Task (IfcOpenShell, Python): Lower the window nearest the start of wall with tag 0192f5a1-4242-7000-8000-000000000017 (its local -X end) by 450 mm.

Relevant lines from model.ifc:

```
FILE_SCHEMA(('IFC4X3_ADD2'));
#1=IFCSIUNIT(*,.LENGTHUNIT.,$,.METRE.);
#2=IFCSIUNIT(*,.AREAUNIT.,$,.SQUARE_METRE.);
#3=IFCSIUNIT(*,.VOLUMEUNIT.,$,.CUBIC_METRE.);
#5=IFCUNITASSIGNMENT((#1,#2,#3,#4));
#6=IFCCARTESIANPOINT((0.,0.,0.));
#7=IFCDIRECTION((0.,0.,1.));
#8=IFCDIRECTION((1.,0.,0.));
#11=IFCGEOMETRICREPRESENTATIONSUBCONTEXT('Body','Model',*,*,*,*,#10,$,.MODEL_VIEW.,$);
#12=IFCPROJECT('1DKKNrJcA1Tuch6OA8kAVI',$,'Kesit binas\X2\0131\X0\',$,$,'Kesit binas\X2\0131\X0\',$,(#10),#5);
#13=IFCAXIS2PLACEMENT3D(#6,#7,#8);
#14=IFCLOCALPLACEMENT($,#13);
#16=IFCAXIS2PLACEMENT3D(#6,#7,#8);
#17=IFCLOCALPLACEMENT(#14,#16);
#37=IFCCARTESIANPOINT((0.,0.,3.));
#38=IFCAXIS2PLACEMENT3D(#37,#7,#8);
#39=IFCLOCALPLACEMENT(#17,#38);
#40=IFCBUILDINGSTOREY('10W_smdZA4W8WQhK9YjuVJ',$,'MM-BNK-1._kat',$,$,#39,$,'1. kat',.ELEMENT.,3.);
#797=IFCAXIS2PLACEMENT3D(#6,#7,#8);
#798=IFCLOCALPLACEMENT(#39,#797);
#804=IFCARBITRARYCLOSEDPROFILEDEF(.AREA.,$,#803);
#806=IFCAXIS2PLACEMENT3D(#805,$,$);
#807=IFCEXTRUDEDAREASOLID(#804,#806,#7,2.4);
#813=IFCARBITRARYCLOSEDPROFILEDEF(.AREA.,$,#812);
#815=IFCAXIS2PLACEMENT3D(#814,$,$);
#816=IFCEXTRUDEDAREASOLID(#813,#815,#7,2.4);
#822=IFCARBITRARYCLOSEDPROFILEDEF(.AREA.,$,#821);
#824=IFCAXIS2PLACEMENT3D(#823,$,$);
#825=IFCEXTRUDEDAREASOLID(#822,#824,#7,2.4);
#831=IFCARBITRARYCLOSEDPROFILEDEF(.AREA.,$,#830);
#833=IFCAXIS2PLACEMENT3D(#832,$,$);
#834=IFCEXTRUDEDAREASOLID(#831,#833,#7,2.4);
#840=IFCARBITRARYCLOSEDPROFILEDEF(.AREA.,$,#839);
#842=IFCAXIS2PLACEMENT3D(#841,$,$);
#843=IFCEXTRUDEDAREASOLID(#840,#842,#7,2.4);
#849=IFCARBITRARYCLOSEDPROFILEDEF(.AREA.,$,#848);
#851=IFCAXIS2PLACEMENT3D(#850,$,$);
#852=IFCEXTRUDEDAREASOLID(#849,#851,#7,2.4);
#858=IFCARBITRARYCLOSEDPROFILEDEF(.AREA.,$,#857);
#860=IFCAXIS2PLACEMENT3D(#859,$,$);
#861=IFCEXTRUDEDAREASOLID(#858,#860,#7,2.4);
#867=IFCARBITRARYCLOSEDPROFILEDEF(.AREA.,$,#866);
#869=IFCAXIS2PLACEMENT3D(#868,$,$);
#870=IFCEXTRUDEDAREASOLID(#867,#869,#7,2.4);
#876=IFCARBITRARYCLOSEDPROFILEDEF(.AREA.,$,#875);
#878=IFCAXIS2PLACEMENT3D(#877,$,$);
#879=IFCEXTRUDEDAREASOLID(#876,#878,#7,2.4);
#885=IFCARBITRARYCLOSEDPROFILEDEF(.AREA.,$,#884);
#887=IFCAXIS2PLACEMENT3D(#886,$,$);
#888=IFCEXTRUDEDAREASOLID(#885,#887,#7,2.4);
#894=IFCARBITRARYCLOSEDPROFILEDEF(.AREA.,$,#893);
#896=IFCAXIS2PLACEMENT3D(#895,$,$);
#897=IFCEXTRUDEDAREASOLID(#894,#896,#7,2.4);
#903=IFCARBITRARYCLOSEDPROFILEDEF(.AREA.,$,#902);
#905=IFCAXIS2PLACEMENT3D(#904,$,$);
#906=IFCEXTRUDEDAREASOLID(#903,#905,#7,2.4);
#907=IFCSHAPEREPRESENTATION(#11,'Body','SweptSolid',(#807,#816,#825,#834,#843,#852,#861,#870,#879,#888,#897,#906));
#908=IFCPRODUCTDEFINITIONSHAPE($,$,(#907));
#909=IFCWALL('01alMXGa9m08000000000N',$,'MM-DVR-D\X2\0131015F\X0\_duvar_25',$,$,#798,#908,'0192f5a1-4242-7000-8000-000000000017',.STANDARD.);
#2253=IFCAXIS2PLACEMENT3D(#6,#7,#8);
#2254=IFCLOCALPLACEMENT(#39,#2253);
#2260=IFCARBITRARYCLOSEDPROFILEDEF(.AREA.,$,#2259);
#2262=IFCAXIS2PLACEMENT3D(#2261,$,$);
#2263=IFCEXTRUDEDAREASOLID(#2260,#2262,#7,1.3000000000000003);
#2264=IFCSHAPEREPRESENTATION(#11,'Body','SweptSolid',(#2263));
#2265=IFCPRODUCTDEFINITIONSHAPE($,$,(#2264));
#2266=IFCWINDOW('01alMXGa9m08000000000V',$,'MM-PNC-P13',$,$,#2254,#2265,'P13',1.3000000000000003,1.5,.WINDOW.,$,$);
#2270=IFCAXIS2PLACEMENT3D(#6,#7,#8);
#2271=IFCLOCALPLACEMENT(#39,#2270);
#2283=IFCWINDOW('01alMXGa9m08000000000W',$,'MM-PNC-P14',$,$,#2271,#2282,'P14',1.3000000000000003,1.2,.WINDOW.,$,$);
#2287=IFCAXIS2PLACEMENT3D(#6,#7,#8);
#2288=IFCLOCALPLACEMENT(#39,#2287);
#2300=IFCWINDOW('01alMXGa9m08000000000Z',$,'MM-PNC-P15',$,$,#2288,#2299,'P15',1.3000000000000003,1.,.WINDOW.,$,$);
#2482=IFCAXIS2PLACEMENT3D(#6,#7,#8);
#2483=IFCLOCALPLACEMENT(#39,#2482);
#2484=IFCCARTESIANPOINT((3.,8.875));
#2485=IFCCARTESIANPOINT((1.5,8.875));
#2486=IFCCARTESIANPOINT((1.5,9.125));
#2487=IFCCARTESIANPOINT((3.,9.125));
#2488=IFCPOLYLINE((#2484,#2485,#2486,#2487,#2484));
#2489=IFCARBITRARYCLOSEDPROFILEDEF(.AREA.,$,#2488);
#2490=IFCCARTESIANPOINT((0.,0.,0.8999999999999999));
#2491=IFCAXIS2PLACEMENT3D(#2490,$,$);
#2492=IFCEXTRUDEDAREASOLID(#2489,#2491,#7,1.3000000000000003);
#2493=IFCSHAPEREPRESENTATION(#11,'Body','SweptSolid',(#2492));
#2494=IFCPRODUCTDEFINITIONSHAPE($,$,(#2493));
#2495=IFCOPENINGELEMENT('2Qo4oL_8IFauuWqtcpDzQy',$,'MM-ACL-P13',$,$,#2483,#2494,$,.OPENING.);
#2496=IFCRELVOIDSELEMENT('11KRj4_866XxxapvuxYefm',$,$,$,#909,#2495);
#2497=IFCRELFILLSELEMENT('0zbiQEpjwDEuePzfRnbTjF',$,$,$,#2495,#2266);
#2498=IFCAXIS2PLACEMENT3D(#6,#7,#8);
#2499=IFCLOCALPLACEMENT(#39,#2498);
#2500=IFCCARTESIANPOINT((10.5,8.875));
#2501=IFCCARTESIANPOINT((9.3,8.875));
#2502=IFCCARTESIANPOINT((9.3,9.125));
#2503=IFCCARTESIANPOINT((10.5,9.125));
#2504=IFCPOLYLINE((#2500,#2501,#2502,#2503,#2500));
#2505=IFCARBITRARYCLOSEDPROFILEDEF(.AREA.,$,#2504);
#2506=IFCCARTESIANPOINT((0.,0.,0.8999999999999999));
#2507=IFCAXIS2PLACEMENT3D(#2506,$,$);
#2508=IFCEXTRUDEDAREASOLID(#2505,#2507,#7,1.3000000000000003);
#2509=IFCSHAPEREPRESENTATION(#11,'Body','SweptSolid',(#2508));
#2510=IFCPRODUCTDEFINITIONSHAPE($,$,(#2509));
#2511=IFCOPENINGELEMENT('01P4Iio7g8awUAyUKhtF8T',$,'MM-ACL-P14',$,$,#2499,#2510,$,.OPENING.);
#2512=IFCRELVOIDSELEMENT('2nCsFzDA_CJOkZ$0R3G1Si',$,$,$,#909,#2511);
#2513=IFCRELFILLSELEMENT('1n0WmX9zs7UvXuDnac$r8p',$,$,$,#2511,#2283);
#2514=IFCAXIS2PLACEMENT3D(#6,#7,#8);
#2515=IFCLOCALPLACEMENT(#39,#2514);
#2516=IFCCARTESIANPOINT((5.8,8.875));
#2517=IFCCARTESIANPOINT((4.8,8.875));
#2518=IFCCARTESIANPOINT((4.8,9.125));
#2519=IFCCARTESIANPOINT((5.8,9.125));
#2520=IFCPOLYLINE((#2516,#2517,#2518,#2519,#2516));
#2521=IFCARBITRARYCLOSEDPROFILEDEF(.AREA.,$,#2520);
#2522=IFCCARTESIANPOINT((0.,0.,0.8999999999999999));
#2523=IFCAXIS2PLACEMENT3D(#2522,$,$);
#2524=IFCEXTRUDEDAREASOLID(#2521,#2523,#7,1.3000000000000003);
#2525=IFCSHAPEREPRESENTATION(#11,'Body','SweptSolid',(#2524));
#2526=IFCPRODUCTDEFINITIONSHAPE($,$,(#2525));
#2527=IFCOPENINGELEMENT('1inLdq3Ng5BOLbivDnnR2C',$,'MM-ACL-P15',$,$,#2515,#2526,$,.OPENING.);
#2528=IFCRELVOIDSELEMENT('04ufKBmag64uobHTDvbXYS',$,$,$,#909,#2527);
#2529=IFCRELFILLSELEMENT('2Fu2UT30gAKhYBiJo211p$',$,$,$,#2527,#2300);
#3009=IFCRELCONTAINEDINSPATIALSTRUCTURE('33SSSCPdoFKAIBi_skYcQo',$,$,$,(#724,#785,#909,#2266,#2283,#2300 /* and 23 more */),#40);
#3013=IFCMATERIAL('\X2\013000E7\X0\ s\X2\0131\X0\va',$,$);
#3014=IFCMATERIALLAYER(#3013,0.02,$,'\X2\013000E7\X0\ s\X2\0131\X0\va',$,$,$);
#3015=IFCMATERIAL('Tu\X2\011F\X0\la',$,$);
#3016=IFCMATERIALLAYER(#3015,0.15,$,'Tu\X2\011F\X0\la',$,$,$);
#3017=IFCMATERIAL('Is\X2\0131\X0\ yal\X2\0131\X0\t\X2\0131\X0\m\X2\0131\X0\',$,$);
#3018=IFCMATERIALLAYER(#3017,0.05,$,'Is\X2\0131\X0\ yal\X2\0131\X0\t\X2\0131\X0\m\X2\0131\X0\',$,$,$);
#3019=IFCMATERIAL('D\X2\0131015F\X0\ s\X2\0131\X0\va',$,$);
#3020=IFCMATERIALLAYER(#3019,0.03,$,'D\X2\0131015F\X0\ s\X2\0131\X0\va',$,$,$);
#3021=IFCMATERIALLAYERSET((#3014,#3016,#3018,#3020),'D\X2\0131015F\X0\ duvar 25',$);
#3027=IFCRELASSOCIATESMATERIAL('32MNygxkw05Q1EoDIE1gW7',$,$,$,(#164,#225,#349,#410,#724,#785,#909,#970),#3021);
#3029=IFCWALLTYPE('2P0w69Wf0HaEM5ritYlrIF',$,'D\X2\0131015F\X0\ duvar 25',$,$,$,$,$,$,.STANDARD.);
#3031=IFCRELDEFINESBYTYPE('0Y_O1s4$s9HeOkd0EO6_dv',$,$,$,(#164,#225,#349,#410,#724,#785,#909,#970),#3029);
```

```python
import numpy as np
import ifcopenshell
import ifcopenshell.api.geometry
import ifcopenshell.util.placement
import ifcopenshell.util.unit

model = ifcopenshell.open("model.ifc")
unit_scale = ifcopenshell.util.unit.calculate_unit_scale(model)

window = model.by_id(2266)
opening = window.FillsVoids[0].RelatingOpeningElement
dz = -0.45 / unit_scale

shift = np.array([0.0, 0.0, dz])
# The window is not placed relative to its opening, so move both.
for product in (opening, window):
    matrix = ifcopenshell.util.placement.get_local_placement(product.ObjectPlacement)
    matrix[:3, 3] += shift
    ifcopenshell.api.geometry.edit_object_placement(model, product=product, matrix=matrix, is_si=False)

print(f"moved by {dz * unit_scale:+.3f} m")

model.write("model_rev.ifc")
```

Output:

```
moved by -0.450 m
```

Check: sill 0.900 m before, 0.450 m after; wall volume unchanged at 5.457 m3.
